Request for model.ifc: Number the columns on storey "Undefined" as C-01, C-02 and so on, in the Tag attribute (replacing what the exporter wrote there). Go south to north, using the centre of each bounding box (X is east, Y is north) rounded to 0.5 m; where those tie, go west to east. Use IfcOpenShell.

First a look at what the model holds.

```python
import ifcopenshell
import ifcopenshell.util.element
import ifcopenshell.util.placement

model = ifcopenshell.open("model.ifc")
print(model.schema)
storey = next(s for s in model.by_type("IfcBuildingStorey") if s.Name == "Undefined")
columns = [e for e in ifcopenshell.util.element.get_decomposition(storey) if e.is_a("IfcColumn")]
for e in sorted(columns, key=lambda e: e.id()):
    origin = ifcopenshell.util.placement.get_local_placement(e.ObjectPlacement)[:3, 3]
    print(e.id(), e.Tag, e.Name, origin.round(2) + 0.0, sep=" | ")
```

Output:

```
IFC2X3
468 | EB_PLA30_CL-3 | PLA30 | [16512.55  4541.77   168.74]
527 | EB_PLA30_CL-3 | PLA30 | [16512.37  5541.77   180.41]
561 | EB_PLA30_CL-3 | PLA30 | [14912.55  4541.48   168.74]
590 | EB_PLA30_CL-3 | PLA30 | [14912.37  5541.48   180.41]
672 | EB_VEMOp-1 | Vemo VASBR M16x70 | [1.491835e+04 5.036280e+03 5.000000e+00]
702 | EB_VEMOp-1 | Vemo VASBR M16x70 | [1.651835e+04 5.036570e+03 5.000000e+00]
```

```python
import ifcopenshell
import ifcopenshell.geom
import ifcopenshell.util.element
import ifcopenshell.util.shape

model = ifcopenshell.open("model.ifc")
settings = ifcopenshell.geom.settings()
settings.set("use-world-coords", True)


def centre(element):
    shape = ifcopenshell.geom.create_shape(settings, element)
    return ifcopenshell.util.shape.get_bbox_centroid(shape.geometry)


storey = next(s for s in model.by_type("IfcBuildingStorey") if s.Name == "Undefined")
columns = [e for e in ifcopenshell.util.element.get_decomposition(storey) if e.is_a("IfcColumn")]

# Insertion points can sit at a corner or the storey origin, so sort by the geometry (in metres).
centres = {e: centre(e) for e in columns}
columns.sort(key=lambda e: (round(centres[e][1] / 0.5), centres[e][0]))

for i, e in enumerate(columns, start=1):
    number = f"C-{i:02d}"
    e.Tag = number
    print(e.id(), number)

model.write("model_v2.ifc")
```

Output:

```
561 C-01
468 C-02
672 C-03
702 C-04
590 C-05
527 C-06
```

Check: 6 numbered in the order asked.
